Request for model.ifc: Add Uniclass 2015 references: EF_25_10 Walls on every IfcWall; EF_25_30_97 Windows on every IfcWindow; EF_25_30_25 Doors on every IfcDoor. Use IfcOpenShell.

First a look at what the model holds.

```python
import ifcopenshell

model = ifcopenshell.open("model.ifc")
print(model.schema)
print("classifications:", [c.Name for c in model.by_type("IfcClassification")])
for ifc_class in ("IfcDoor", "IfcRoof", "IfcStair", "IfcWall", "IfcWindow"):
    print(ifc_class, len(model.by_type(ifc_class)))
```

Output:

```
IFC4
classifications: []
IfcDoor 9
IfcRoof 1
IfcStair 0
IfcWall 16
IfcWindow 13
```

```python
import ifcopenshell
import ifcopenshell.api.classification

model = ifcopenshell.open("model.ifc")

system = ifcopenshell.api.classification.add_classification(model, classification="Uniclass 2015")

codes = {
    "IfcWall": ("EF_25_10", "Walls"),
    "IfcWindow": ("EF_25_30_97", "Windows"),
    "IfcDoor": ("EF_25_30_25", "Doors"),
}
for ifc_class, (code, name) in codes.items():
    products = model.by_type(ifc_class)
    ifcopenshell.api.classification.add_reference(
        model, products=products, classification=system, identification=code, name=name
    )
    print(code, len(products))

model.write("model_updated.ifc")
```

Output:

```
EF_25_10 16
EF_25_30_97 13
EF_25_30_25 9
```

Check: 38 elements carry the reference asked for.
